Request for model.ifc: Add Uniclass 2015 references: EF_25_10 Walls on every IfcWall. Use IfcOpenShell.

First a look at what the model holds.

```python
import ifcopenshell

model = ifcopenshell.open("model.ifc")
print(model.schema)
print("classifications:", [c.Name for c in model.by_type("IfcClassification")])
for ifc_class in ("IfcDoor", "IfcRoof", "IfcStair", "IfcWall", "IfcWindow"):
    print(ifc_class, len(model.by_type(ifc_class)))
```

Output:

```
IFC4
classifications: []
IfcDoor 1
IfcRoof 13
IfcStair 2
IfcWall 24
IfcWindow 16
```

```python
import ifcopenshell
import ifcopenshell.api.classification

model = ifcopenshell.open("model.ifc")

system = ifcopenshell.api.classification.add_classification(model, classification="Uniclass 2015")

codes = {
    "IfcWall": ("EF_25_10", "Walls"),
}
for ifc_class, (code, name) in codes.items():
    products = model.by_type(ifc_class)
    ifcopenshell.api.classification.add_reference(
        model, products=products, classification=system, identification=code, name=name
    )
    print(code, len(products))

model.write("model_rev.ifc")
```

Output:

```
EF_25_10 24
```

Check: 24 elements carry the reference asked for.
